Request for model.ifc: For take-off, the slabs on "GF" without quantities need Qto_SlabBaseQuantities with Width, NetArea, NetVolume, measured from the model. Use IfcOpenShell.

First a look at what the model holds.

```python
import ifcopenshell
import ifcopenshell.util.element
import ifcopenshell.util.unit

model = ifcopenshell.open("model.ifc")
print(model.schema)
for unit_type in ("LENGTHUNIT", "AREAUNIT", "VOLUMEUNIT"):
    print(unit_type, ifcopenshell.util.unit.calculate_unit_scale(model, unit_type))
storey = next(s for s in model.by_type("IfcBuildingStorey") if s.Name == "GF")
slabs = [e for e in ifcopenshell.util.element.get_decomposition(storey) if e.is_a("IfcSlab")]
for e in sorted(slabs, key=lambda e: e.id()):
    print(e.id(), e.is_a(), e.Name, list(ifcopenshell.util.element.get_psets(e, qtos_only=True)), sep=" | ")
```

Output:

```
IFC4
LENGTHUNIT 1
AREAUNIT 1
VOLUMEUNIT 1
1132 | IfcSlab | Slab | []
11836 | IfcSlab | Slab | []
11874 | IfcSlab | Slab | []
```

```python
import ifcopenshell
import ifcopenshell.api.pset
import ifcopenshell.geom
import ifcopenshell.util.element
import ifcopenshell.util.shape
import ifcopenshell.util.unit

model = ifcopenshell.open("model.ifc")
unit_scale = ifcopenshell.util.unit.calculate_unit_scale(model)
area_scale = ifcopenshell.util.unit.calculate_unit_scale(model, "AREAUNIT")
volume_scale = ifcopenshell.util.unit.calculate_unit_scale(model, "VOLUMEUNIT")
settings = ifcopenshell.geom.settings()

storey = next(s for s in model.by_type("IfcBuildingStorey") if s.Name == "GF")
slabs = [e for e in ifcopenshell.util.element.get_decomposition(storey) if e.is_a("IfcSlab")]

for e in sorted(slabs, key=lambda e: e.id()):
    if ifcopenshell.util.element.get_psets(e, qtos_only=True, should_inherit=False):
        continue
    # Geometry comes back in metres, in the element's own axes.
    shape = ifcopenshell.geom.create_shape(settings, e)
    values = {
        "Width": ifcopenshell.util.shape.get_z(shape.geometry) / unit_scale,
        "NetArea": ifcopenshell.util.shape.get_footprint_area(shape.geometry) / area_scale,
        "NetVolume": ifcopenshell.util.shape.get_volume(shape.geometry) / volume_scale,
    }
    qto = ifcopenshell.api.pset.add_qto(model, product=e, name="Qto_SlabBaseQuantities")
    ifcopenshell.api.pset.edit_qto(model, qto=qto, properties=values)
    print(e.id(), {k: round(v, 3) for k, v in values.items()})

model.write("model_v2.ifc")
```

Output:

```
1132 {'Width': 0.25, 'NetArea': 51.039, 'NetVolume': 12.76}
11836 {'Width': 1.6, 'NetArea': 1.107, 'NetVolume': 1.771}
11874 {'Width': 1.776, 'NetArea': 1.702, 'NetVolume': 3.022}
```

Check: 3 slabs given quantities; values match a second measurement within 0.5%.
